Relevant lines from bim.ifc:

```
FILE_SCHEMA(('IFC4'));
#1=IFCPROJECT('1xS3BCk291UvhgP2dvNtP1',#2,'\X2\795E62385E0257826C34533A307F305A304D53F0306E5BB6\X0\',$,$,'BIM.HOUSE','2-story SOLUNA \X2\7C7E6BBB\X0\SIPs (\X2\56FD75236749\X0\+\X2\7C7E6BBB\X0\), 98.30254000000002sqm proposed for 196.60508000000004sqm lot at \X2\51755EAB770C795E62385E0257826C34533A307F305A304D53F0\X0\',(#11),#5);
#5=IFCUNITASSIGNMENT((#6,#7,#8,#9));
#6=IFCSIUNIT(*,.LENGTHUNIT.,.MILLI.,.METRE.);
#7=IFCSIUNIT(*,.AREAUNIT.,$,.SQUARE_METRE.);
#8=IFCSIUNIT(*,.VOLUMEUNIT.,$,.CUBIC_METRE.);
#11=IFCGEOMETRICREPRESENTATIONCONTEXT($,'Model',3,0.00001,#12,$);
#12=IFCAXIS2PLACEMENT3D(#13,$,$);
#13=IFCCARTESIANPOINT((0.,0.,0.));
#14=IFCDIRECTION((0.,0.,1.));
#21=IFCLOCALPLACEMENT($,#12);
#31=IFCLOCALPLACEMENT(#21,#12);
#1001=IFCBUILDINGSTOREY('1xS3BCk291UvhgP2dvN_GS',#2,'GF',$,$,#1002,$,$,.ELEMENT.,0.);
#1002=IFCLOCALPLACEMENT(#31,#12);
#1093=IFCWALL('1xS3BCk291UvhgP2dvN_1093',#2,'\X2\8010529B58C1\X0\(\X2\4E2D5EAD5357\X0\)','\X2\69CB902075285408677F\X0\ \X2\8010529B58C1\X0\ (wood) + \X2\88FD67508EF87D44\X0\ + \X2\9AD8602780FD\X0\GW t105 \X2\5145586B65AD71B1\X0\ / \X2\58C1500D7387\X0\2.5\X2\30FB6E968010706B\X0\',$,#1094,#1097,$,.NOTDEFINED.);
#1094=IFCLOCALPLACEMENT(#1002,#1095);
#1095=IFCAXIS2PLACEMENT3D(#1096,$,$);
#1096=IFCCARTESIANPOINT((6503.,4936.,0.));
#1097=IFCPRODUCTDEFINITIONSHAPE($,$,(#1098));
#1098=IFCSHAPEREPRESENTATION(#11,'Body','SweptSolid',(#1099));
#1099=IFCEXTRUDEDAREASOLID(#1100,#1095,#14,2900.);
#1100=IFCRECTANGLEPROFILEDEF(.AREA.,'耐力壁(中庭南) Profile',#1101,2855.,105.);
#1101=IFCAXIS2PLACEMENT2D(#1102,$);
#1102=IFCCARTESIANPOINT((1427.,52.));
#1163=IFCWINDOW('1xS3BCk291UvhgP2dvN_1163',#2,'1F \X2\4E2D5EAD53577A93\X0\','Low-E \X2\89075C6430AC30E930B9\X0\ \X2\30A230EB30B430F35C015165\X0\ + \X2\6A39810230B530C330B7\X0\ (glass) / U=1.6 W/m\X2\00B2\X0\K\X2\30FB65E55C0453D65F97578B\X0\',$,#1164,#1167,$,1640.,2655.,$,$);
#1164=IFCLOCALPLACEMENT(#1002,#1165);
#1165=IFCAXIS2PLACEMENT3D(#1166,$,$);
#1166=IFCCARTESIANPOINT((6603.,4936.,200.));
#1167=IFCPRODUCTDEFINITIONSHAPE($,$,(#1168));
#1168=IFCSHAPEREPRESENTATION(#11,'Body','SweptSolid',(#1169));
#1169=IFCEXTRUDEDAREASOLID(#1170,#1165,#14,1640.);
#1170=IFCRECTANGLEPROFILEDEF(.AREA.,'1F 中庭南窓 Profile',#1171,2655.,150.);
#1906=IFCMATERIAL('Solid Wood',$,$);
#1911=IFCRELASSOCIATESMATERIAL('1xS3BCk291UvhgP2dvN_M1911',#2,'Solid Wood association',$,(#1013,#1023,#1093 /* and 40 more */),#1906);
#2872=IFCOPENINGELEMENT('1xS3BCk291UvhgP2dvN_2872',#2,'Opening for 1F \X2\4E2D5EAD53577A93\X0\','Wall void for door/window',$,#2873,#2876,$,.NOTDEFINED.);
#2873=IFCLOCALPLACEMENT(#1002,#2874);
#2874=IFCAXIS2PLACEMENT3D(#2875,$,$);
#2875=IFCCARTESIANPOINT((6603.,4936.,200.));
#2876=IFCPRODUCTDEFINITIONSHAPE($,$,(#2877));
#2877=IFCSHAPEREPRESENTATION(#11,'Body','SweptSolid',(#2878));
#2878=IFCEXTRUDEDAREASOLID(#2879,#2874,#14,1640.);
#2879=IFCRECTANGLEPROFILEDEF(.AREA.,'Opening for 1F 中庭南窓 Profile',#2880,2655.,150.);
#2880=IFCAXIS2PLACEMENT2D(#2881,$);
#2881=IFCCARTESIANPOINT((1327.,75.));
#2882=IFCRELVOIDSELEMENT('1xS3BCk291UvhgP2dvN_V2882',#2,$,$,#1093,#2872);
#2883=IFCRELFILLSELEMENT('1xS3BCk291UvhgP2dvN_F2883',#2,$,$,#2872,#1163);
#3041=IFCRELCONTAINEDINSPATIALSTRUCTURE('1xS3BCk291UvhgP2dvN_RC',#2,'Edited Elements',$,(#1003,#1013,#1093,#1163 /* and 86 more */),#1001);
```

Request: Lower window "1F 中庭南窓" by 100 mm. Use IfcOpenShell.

```python
import numpy as np
import ifcopenshell
import ifcopenshell.api.geometry
import ifcopenshell.util.placement
import ifcopenshell.util.unit

model = ifcopenshell.open("bim.ifc")
unit_scale = ifcopenshell.util.unit.calculate_unit_scale(model)

window = model.by_guid("1xS3BCk291UvhgP2dvN_1163")
opening = window.FillsVoids[0].RelatingOpeningElement
dz = -100.0

shift = np.array([0.0, 0.0, dz])
# The window is not placed relative to its opening, so move both.
for product in (opening, window):
    matrix = ifcopenshell.util.placement.get_local_placement(product.ObjectPlacement)
    matrix[:3, 3] += shift
    ifcopenshell.api.geometry.edit_object_placement(model, product=product, matrix=matrix, is_si=False)

print(f"moved by {dz * unit_scale:+.3f} m")

model.write("bim_edited.ifc")
```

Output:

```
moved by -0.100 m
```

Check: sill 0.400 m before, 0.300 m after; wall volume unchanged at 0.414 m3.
